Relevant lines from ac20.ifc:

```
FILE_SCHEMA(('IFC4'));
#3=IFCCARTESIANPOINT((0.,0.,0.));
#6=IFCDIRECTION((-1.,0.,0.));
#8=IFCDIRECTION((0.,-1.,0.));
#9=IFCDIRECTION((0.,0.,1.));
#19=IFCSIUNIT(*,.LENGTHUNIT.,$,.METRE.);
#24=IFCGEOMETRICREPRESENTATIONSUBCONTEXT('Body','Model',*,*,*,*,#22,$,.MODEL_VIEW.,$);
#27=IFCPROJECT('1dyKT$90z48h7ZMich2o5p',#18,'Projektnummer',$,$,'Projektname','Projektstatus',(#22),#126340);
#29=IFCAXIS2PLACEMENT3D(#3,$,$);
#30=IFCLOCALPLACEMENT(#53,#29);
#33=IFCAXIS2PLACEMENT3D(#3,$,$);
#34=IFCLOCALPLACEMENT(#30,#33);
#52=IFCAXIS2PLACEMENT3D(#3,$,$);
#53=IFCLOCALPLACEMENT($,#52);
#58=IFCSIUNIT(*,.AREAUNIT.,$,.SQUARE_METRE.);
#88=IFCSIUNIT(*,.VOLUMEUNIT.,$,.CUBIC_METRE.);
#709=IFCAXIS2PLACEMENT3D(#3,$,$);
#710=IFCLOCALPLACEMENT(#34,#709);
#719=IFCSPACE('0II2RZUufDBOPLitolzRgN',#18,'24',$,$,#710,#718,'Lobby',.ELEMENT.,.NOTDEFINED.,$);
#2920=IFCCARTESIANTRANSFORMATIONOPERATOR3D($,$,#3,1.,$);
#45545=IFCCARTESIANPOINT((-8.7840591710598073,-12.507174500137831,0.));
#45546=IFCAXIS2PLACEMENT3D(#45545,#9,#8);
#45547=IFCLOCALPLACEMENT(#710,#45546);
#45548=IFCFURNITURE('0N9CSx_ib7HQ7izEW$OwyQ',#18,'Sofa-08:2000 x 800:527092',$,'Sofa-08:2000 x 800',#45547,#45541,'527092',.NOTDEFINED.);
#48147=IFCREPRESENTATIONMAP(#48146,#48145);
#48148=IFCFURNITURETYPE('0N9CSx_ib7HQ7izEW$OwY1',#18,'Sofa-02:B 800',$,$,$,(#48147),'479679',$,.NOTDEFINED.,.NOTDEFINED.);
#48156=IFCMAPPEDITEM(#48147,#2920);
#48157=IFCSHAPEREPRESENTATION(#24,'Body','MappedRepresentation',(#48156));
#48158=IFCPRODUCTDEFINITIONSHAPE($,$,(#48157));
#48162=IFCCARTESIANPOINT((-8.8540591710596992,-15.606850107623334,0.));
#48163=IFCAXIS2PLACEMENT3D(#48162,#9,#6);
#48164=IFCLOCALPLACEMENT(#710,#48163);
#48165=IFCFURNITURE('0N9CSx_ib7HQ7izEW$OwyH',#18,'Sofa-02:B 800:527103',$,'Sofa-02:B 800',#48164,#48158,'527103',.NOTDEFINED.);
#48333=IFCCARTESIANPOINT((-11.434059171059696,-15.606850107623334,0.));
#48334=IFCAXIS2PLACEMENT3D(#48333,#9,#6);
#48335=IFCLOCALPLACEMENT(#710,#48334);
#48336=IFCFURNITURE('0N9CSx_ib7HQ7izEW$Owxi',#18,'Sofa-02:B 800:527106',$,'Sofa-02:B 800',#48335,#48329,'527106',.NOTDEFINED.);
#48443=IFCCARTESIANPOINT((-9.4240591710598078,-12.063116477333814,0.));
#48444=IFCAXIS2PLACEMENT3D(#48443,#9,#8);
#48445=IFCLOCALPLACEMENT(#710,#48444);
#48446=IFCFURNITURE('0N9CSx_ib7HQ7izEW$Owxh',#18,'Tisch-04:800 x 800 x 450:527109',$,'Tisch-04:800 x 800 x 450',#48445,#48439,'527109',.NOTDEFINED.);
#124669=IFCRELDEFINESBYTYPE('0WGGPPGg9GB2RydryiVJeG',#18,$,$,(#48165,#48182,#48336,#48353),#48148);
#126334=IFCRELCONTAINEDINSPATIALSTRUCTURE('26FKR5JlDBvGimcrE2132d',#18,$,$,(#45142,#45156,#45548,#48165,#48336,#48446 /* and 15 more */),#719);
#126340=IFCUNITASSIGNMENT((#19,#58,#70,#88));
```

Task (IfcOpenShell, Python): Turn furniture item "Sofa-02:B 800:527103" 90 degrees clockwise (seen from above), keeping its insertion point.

```python
import ifcopenshell
import ifcopenshell.api.geometry
import ifcopenshell.util.placement

model = ifcopenshell.open("ac20.ifc")

item = model.by_guid("0N9CSx_ib7HQ7izEW$OwyH")
matrix = ifcopenshell.util.placement.get_local_placement(item.ObjectPlacement)
matrix = matrix @ ifcopenshell.util.placement.rotation(-90, "Z")
ifcopenshell.api.geometry.edit_object_placement(model, product=item, matrix=matrix, is_si=False)

print(ifcopenshell.util.placement.get_local_placement(item.ObjectPlacement).round(3) + 0.0)

model.write("ac20_rev.ifc")
```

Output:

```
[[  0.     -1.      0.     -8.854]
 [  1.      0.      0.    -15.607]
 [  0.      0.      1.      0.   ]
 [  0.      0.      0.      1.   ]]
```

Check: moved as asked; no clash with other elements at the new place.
